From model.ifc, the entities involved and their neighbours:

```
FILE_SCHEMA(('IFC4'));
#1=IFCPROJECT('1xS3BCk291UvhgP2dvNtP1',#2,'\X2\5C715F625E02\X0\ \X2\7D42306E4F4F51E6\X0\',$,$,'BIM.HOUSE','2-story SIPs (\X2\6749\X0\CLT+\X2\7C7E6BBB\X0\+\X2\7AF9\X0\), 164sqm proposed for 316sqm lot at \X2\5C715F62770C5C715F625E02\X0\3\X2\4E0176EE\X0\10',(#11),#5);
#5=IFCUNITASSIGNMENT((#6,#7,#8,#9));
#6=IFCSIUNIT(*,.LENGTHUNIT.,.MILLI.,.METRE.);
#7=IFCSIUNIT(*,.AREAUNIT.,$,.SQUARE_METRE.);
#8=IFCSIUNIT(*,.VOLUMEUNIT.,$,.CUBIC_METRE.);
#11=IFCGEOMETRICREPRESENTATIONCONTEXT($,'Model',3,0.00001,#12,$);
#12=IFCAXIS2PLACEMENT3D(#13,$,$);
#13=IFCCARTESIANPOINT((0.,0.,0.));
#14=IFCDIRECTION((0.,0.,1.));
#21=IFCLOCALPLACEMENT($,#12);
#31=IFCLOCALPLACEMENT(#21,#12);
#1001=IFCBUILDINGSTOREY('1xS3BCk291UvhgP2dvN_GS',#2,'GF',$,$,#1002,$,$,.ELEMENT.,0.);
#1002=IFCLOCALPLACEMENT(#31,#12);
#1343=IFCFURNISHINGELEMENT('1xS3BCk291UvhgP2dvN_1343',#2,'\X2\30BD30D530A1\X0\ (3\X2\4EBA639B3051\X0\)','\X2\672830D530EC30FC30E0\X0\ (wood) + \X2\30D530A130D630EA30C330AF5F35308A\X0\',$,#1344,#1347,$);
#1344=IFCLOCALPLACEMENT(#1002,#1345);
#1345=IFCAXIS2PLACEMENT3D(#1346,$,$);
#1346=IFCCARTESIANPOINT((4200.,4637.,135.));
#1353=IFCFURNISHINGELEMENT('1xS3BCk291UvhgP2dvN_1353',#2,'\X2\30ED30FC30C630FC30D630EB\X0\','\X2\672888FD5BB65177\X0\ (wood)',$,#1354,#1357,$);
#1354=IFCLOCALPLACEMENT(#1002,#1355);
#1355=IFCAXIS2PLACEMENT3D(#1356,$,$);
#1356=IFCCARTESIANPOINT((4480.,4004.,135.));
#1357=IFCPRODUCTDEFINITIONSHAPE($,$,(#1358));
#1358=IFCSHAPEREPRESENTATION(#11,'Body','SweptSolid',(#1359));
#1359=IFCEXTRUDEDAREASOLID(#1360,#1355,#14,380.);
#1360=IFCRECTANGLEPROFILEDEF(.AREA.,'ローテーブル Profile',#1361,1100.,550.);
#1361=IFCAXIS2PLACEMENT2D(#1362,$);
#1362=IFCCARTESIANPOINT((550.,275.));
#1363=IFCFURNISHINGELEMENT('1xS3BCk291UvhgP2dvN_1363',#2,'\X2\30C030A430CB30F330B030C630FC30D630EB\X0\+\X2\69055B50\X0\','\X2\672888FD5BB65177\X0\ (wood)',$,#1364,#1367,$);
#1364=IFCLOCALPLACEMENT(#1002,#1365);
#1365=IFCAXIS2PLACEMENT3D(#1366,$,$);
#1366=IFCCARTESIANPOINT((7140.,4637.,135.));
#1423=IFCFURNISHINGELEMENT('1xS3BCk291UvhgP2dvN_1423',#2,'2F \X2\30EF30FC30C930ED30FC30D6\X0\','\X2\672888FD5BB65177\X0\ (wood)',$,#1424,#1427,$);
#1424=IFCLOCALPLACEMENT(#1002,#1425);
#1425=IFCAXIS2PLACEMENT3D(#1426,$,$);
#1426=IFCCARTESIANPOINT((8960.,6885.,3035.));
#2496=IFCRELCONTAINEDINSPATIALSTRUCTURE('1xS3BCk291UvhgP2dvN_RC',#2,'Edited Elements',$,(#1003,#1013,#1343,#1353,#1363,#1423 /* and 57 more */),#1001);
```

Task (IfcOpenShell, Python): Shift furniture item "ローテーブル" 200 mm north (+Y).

```python
import ifcopenshell
import ifcopenshell.api.geometry
import ifcopenshell.util.placement

model = ifcopenshell.open("model.ifc")

item = model.by_guid("1xS3BCk291UvhgP2dvN_1353")
matrix = ifcopenshell.util.placement.get_local_placement(item.ObjectPlacement)
matrix[1, 3] += 200.0
ifcopenshell.api.geometry.edit_object_placement(model, product=item, matrix=matrix, is_si=False)

print(ifcopenshell.util.placement.get_local_placement(item.ObjectPlacement).round(3) + 0.0)

model.write("model_v2.ifc")
```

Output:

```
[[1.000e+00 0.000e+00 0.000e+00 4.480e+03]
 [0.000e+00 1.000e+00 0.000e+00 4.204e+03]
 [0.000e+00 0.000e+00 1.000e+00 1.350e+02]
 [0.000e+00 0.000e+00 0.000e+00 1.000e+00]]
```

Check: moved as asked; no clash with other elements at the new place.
